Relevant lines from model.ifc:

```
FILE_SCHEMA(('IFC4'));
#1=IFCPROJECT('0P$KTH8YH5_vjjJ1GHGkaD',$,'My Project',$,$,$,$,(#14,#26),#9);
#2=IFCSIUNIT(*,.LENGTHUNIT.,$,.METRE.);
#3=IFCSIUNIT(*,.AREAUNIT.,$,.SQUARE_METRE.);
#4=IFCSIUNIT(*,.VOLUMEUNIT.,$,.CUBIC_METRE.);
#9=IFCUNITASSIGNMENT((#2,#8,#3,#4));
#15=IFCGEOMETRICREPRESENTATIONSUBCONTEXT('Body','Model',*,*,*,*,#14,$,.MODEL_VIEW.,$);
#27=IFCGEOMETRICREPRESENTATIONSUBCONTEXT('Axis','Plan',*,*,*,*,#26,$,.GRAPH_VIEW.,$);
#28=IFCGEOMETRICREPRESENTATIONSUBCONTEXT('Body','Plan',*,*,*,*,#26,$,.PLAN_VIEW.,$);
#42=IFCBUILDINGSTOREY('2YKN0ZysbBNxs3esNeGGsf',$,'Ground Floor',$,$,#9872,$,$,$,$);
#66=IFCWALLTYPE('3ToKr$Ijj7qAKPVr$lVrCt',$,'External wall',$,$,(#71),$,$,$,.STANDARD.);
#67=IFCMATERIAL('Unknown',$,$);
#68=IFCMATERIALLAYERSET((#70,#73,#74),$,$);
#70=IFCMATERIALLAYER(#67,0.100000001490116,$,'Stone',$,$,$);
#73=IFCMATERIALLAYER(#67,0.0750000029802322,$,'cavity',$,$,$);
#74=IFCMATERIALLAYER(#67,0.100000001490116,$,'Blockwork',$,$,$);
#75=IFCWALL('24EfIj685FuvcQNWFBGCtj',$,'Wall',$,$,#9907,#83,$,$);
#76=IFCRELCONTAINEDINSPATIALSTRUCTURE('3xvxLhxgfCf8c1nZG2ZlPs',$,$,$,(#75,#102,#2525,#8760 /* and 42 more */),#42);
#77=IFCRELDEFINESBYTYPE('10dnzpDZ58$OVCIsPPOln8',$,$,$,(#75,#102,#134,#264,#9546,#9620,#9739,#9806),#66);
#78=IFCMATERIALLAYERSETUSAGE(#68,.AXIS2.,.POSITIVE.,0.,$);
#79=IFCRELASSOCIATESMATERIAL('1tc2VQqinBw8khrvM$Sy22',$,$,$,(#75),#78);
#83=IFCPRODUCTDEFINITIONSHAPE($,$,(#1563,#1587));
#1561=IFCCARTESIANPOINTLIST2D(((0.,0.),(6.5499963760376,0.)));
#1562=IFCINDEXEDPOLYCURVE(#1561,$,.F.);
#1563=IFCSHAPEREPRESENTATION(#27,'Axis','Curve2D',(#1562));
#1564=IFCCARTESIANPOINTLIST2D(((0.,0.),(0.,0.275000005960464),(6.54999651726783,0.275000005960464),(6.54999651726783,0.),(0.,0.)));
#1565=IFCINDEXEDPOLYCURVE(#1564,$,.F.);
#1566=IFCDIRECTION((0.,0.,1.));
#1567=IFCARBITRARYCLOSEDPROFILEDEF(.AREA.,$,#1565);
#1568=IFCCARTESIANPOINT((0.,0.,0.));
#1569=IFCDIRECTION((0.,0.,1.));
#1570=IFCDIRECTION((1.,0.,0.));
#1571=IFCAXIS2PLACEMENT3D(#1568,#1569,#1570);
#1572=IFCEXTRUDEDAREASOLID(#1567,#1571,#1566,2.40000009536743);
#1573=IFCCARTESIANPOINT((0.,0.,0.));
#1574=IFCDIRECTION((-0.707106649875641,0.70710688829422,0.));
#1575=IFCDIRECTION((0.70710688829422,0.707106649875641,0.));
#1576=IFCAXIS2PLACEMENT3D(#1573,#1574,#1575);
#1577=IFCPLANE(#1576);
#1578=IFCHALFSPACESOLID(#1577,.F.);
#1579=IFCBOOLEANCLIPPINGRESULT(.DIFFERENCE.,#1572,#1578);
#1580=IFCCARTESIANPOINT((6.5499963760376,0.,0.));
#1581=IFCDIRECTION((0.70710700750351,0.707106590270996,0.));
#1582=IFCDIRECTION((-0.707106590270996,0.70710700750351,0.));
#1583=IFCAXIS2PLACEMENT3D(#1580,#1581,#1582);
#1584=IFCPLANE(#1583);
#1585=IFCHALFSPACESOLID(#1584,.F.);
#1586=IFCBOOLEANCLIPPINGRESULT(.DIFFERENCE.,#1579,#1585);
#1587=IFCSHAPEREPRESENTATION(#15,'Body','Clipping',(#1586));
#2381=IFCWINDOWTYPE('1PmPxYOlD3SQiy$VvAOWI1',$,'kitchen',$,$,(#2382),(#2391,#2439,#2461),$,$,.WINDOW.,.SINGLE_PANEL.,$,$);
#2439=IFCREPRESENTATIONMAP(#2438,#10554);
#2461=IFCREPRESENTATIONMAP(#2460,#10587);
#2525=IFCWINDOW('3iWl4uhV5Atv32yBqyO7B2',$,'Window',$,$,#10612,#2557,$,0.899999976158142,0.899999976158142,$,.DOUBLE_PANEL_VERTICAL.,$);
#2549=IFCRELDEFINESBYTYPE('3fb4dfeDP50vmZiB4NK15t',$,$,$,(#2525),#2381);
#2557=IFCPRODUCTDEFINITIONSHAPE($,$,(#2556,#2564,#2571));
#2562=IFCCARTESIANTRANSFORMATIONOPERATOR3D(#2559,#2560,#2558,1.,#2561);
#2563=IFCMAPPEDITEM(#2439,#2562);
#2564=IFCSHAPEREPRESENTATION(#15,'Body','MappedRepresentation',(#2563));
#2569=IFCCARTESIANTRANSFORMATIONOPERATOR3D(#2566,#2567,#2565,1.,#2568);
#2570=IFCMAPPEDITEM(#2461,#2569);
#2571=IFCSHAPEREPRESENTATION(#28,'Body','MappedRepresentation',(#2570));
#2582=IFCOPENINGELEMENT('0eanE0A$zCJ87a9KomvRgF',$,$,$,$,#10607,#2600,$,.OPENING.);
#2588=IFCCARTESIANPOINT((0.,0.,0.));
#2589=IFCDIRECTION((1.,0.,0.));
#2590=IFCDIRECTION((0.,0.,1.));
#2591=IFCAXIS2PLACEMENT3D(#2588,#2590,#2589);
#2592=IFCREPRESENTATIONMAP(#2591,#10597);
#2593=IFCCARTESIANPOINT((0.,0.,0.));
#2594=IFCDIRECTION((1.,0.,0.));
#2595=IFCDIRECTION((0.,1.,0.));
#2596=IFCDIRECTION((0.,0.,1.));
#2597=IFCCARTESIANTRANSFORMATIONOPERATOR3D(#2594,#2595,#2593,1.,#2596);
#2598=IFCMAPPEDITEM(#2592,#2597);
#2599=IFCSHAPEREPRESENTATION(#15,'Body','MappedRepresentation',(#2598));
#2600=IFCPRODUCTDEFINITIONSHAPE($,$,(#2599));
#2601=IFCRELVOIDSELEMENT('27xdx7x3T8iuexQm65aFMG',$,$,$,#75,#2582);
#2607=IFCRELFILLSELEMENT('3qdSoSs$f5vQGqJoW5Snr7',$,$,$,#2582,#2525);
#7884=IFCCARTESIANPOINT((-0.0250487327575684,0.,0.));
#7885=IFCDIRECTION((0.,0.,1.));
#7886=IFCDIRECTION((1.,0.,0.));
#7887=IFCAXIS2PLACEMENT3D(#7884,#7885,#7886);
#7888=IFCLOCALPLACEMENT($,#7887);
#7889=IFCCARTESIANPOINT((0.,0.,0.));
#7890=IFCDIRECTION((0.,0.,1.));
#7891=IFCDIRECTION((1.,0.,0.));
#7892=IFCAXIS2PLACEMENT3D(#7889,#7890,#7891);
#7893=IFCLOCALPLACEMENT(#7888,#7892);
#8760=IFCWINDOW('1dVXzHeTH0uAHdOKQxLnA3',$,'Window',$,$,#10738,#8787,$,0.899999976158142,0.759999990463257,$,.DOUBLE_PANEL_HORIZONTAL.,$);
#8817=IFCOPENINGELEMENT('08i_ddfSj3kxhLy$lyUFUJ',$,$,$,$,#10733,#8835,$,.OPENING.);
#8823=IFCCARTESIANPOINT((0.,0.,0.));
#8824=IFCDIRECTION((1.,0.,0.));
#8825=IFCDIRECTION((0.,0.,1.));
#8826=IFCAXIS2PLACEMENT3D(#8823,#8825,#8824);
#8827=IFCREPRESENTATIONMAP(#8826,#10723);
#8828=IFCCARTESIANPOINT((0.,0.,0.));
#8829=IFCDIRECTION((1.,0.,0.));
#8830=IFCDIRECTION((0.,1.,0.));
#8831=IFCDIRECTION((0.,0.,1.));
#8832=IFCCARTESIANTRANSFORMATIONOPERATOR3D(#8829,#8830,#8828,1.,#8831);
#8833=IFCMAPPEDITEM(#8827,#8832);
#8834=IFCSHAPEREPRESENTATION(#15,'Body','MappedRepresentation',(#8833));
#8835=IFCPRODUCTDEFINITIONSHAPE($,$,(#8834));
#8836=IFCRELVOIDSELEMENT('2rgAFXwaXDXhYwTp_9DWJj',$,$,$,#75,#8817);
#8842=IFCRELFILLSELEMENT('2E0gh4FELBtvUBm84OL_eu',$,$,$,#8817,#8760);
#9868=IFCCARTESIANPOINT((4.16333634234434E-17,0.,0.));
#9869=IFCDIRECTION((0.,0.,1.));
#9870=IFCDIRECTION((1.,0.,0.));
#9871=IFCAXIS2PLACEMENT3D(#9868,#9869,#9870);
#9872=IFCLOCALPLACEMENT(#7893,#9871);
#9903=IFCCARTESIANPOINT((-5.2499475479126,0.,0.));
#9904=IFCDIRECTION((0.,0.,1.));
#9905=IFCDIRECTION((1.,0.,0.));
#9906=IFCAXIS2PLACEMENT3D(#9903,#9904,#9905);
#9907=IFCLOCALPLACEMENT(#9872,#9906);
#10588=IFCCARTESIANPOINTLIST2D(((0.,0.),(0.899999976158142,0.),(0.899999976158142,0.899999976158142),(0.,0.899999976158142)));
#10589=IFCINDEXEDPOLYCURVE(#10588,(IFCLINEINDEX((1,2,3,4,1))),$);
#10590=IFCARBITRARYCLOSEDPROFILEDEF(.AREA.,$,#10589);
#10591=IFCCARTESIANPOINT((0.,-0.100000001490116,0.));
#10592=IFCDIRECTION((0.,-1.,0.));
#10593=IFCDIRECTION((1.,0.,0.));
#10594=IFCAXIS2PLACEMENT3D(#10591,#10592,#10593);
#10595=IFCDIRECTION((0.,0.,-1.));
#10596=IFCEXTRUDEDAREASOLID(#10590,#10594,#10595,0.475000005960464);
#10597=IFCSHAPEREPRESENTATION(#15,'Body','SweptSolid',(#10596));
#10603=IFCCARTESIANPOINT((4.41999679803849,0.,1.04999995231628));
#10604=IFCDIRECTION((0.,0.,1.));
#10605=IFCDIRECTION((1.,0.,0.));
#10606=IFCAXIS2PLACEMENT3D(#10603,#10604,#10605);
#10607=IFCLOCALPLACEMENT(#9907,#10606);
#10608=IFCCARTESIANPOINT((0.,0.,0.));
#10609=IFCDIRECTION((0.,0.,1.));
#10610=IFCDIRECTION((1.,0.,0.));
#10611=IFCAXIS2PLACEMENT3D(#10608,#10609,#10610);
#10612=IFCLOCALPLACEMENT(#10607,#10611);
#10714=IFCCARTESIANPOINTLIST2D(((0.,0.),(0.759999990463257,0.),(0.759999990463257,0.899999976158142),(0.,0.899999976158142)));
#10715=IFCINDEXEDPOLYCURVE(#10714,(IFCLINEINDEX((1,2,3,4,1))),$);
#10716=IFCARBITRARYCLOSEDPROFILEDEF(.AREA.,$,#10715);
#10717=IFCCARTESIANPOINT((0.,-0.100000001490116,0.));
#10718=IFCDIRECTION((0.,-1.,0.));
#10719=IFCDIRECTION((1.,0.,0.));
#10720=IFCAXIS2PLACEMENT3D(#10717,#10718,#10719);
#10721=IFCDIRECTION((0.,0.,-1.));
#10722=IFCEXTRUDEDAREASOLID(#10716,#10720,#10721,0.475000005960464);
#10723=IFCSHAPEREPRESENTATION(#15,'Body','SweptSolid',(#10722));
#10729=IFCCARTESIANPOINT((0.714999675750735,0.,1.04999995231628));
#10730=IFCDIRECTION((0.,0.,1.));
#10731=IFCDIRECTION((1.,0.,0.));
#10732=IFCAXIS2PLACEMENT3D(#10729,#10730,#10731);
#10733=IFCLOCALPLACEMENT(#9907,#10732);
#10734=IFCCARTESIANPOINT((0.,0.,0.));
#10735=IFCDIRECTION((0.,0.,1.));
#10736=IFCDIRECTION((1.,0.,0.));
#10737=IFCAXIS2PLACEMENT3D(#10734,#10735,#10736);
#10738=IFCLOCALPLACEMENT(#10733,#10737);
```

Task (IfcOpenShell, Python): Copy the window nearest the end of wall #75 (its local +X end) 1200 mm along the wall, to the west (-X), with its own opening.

```python
import ifcopenshell
import ifcopenshell.api.feature
import ifcopenshell.api.geometry
import ifcopenshell.api.root
import ifcopenshell.geom
import ifcopenshell.util.element
import ifcopenshell.util.placement
import ifcopenshell.util.shape
import ifcopenshell.util.unit

model = ifcopenshell.open("model.ifc")
unit_scale = ifcopenshell.util.unit.calculate_unit_scale(model)
settings = ifcopenshell.geom.settings()


def volume(element):
    """Net volume in cubic metres, openings subtracted."""
    shape = ifcopenshell.geom.create_shape(settings, element)
    return ifcopenshell.util.shape.get_volume(shape.geometry)


window = model.by_guid("3iWl4uhV5Atv32yBqyO7B2")
opening = window.FillsVoids[0].RelatingOpeningElement
wall = opening.VoidsElements[0].RelatingBuildingElement
before = volume(wall)
shift = ifcopenshell.util.placement.get_local_placement(wall.ObjectPlacement)[:3, 0] * -1.2 / unit_scale

# copy_class copies the void relationship, type, container and properties, but no geometry.
new_opening = ifcopenshell.api.root.copy_class(model, product=opening)
new_opening.Representation = ifcopenshell.util.element.copy_deep(
    model, opening.Representation, exclude=["IfcGeometricRepresentationContext", "IfcRepresentationMap"]
)
new_window = ifcopenshell.api.root.copy_class(model, product=window)
new_window.Representation = ifcopenshell.util.element.copy_deep(
    model, window.Representation, exclude=["IfcGeometricRepresentationContext", "IfcRepresentationMap"]
)
ifcopenshell.api.feature.add_filling(model, opening=new_opening, element=new_window)

for old, new in ((opening, new_opening), (window, new_window)):
    matrix = ifcopenshell.util.placement.get_local_placement(old.ObjectPlacement)
    matrix[:3, 3] += shift
    ifcopenshell.api.geometry.edit_object_placement(model, product=new, matrix=matrix, is_si=False)

after = volume(wall)

print(f"wall volume {before:.3f} -> {after:.3f} m3")

model.write("model-out.ifc")
```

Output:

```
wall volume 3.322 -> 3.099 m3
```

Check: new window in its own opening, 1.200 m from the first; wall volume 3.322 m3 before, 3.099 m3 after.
